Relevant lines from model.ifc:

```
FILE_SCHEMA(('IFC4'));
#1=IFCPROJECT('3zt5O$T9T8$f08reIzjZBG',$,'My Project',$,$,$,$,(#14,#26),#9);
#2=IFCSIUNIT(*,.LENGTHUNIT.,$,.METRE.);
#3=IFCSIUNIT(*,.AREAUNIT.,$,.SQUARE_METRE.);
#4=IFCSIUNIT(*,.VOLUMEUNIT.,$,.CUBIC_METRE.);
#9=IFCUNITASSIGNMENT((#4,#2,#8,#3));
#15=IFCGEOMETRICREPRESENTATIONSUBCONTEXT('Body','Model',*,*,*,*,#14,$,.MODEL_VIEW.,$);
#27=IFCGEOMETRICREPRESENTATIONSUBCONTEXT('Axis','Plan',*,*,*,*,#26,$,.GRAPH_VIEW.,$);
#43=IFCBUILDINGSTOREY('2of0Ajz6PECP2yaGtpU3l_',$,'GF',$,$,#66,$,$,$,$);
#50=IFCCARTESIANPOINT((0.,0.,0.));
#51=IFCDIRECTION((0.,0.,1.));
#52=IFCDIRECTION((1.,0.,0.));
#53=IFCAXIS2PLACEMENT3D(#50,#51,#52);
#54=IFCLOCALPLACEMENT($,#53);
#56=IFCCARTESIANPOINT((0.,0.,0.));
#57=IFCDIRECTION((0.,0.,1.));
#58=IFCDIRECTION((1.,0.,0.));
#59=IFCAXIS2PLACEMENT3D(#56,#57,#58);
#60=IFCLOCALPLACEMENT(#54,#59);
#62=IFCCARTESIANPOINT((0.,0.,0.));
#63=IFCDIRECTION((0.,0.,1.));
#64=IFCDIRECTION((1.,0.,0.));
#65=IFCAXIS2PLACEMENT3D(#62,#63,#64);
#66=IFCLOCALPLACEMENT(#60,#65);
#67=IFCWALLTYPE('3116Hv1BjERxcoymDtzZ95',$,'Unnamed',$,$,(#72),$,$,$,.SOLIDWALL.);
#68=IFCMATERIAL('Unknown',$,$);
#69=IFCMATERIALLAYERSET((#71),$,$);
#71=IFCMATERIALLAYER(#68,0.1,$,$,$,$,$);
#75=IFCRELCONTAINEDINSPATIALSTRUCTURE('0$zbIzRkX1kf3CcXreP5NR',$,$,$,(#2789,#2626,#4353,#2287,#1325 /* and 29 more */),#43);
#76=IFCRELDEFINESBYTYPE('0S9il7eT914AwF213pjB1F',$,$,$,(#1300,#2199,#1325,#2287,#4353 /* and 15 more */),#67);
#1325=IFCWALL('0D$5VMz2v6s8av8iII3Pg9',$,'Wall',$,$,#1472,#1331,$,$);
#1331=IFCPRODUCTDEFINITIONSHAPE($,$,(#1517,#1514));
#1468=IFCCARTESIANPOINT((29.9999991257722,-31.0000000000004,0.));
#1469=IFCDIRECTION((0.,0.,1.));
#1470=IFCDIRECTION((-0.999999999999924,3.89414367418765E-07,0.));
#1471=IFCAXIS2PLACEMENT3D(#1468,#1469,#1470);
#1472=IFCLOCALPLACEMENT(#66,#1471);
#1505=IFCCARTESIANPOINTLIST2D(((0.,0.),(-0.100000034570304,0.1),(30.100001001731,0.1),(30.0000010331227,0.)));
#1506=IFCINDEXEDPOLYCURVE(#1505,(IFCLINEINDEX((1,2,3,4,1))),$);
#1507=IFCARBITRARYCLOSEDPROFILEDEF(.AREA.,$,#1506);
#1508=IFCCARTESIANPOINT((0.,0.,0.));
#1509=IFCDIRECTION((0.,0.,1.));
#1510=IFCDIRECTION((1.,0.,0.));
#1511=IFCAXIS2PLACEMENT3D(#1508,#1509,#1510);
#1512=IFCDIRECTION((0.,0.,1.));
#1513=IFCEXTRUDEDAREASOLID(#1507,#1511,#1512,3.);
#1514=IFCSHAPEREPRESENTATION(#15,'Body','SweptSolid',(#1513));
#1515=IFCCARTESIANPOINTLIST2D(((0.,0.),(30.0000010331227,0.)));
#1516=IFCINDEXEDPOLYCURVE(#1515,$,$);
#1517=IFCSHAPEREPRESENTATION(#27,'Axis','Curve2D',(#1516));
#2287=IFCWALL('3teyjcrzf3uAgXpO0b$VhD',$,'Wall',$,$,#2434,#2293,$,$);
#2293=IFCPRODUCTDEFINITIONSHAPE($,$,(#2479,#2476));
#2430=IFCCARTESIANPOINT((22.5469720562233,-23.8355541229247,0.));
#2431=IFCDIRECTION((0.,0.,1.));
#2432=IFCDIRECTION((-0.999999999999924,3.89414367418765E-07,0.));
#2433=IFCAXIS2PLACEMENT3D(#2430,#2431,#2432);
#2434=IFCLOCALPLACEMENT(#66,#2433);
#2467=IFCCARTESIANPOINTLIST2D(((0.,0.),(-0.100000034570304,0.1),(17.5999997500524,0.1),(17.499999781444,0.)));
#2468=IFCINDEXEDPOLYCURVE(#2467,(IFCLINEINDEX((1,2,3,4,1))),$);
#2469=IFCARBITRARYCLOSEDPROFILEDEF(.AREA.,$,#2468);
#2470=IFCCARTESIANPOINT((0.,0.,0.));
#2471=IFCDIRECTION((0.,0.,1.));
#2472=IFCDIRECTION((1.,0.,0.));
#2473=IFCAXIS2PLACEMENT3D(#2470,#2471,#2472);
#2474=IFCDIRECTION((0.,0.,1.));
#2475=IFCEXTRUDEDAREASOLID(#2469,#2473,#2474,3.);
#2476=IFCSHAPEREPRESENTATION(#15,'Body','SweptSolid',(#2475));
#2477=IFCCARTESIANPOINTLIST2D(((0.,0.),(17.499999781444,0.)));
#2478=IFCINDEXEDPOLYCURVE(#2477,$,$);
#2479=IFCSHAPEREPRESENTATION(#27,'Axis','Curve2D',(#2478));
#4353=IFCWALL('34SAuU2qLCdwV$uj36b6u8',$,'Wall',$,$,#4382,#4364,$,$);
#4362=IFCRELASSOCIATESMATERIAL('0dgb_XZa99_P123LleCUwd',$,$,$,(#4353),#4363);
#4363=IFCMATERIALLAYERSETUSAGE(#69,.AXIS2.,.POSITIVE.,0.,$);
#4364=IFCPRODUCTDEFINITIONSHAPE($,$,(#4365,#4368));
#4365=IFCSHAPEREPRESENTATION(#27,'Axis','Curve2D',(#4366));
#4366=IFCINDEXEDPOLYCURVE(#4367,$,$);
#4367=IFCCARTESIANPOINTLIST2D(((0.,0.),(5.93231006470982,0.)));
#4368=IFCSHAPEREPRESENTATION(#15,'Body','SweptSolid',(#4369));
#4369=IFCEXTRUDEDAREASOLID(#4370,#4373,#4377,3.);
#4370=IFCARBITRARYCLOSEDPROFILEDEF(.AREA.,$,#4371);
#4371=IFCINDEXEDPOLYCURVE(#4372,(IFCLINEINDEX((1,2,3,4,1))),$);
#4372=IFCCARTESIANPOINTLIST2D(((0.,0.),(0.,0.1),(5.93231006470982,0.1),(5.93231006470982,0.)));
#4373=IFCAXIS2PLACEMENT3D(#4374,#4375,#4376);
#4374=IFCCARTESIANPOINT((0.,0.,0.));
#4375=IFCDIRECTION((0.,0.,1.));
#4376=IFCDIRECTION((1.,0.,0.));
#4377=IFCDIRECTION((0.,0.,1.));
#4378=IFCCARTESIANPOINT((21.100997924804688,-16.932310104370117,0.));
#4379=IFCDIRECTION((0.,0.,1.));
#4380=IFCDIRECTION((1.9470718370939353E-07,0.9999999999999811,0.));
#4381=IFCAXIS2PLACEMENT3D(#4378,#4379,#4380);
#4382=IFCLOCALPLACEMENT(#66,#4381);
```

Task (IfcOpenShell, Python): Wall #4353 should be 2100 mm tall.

```python
import ifcopenshell
import ifcopenshell.geom
import ifcopenshell.util.representation
import ifcopenshell.util.shape
import ifcopenshell.util.unit

model = ifcopenshell.open("model.ifc")
unit_scale = ifcopenshell.util.unit.calculate_unit_scale(model)
settings = ifcopenshell.geom.settings()


def volume(element):
    """Net volume in cubic metres, openings subtracted."""
    shape = ifcopenshell.geom.create_shape(settings, element)
    return ifcopenshell.util.shape.get_volume(shape.geometry)


wall = model.by_guid("34SAuU2qLCdwV$uj36b6u8")
before = volume(wall)

body = ifcopenshell.util.representation.get_representation(wall, "Model", "Body")
solid = body.Items[0]
old_height = solid.Depth
solid.Depth = 2.1 / unit_scale
after = volume(wall)

print(f"height {old_height:g} -> {solid.Depth:g}, volume {before:.3f} -> {after:.3f} m3")

model.write("model_v2.ifc")
```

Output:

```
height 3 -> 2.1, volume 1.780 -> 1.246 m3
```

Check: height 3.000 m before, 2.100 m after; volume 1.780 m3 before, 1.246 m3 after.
